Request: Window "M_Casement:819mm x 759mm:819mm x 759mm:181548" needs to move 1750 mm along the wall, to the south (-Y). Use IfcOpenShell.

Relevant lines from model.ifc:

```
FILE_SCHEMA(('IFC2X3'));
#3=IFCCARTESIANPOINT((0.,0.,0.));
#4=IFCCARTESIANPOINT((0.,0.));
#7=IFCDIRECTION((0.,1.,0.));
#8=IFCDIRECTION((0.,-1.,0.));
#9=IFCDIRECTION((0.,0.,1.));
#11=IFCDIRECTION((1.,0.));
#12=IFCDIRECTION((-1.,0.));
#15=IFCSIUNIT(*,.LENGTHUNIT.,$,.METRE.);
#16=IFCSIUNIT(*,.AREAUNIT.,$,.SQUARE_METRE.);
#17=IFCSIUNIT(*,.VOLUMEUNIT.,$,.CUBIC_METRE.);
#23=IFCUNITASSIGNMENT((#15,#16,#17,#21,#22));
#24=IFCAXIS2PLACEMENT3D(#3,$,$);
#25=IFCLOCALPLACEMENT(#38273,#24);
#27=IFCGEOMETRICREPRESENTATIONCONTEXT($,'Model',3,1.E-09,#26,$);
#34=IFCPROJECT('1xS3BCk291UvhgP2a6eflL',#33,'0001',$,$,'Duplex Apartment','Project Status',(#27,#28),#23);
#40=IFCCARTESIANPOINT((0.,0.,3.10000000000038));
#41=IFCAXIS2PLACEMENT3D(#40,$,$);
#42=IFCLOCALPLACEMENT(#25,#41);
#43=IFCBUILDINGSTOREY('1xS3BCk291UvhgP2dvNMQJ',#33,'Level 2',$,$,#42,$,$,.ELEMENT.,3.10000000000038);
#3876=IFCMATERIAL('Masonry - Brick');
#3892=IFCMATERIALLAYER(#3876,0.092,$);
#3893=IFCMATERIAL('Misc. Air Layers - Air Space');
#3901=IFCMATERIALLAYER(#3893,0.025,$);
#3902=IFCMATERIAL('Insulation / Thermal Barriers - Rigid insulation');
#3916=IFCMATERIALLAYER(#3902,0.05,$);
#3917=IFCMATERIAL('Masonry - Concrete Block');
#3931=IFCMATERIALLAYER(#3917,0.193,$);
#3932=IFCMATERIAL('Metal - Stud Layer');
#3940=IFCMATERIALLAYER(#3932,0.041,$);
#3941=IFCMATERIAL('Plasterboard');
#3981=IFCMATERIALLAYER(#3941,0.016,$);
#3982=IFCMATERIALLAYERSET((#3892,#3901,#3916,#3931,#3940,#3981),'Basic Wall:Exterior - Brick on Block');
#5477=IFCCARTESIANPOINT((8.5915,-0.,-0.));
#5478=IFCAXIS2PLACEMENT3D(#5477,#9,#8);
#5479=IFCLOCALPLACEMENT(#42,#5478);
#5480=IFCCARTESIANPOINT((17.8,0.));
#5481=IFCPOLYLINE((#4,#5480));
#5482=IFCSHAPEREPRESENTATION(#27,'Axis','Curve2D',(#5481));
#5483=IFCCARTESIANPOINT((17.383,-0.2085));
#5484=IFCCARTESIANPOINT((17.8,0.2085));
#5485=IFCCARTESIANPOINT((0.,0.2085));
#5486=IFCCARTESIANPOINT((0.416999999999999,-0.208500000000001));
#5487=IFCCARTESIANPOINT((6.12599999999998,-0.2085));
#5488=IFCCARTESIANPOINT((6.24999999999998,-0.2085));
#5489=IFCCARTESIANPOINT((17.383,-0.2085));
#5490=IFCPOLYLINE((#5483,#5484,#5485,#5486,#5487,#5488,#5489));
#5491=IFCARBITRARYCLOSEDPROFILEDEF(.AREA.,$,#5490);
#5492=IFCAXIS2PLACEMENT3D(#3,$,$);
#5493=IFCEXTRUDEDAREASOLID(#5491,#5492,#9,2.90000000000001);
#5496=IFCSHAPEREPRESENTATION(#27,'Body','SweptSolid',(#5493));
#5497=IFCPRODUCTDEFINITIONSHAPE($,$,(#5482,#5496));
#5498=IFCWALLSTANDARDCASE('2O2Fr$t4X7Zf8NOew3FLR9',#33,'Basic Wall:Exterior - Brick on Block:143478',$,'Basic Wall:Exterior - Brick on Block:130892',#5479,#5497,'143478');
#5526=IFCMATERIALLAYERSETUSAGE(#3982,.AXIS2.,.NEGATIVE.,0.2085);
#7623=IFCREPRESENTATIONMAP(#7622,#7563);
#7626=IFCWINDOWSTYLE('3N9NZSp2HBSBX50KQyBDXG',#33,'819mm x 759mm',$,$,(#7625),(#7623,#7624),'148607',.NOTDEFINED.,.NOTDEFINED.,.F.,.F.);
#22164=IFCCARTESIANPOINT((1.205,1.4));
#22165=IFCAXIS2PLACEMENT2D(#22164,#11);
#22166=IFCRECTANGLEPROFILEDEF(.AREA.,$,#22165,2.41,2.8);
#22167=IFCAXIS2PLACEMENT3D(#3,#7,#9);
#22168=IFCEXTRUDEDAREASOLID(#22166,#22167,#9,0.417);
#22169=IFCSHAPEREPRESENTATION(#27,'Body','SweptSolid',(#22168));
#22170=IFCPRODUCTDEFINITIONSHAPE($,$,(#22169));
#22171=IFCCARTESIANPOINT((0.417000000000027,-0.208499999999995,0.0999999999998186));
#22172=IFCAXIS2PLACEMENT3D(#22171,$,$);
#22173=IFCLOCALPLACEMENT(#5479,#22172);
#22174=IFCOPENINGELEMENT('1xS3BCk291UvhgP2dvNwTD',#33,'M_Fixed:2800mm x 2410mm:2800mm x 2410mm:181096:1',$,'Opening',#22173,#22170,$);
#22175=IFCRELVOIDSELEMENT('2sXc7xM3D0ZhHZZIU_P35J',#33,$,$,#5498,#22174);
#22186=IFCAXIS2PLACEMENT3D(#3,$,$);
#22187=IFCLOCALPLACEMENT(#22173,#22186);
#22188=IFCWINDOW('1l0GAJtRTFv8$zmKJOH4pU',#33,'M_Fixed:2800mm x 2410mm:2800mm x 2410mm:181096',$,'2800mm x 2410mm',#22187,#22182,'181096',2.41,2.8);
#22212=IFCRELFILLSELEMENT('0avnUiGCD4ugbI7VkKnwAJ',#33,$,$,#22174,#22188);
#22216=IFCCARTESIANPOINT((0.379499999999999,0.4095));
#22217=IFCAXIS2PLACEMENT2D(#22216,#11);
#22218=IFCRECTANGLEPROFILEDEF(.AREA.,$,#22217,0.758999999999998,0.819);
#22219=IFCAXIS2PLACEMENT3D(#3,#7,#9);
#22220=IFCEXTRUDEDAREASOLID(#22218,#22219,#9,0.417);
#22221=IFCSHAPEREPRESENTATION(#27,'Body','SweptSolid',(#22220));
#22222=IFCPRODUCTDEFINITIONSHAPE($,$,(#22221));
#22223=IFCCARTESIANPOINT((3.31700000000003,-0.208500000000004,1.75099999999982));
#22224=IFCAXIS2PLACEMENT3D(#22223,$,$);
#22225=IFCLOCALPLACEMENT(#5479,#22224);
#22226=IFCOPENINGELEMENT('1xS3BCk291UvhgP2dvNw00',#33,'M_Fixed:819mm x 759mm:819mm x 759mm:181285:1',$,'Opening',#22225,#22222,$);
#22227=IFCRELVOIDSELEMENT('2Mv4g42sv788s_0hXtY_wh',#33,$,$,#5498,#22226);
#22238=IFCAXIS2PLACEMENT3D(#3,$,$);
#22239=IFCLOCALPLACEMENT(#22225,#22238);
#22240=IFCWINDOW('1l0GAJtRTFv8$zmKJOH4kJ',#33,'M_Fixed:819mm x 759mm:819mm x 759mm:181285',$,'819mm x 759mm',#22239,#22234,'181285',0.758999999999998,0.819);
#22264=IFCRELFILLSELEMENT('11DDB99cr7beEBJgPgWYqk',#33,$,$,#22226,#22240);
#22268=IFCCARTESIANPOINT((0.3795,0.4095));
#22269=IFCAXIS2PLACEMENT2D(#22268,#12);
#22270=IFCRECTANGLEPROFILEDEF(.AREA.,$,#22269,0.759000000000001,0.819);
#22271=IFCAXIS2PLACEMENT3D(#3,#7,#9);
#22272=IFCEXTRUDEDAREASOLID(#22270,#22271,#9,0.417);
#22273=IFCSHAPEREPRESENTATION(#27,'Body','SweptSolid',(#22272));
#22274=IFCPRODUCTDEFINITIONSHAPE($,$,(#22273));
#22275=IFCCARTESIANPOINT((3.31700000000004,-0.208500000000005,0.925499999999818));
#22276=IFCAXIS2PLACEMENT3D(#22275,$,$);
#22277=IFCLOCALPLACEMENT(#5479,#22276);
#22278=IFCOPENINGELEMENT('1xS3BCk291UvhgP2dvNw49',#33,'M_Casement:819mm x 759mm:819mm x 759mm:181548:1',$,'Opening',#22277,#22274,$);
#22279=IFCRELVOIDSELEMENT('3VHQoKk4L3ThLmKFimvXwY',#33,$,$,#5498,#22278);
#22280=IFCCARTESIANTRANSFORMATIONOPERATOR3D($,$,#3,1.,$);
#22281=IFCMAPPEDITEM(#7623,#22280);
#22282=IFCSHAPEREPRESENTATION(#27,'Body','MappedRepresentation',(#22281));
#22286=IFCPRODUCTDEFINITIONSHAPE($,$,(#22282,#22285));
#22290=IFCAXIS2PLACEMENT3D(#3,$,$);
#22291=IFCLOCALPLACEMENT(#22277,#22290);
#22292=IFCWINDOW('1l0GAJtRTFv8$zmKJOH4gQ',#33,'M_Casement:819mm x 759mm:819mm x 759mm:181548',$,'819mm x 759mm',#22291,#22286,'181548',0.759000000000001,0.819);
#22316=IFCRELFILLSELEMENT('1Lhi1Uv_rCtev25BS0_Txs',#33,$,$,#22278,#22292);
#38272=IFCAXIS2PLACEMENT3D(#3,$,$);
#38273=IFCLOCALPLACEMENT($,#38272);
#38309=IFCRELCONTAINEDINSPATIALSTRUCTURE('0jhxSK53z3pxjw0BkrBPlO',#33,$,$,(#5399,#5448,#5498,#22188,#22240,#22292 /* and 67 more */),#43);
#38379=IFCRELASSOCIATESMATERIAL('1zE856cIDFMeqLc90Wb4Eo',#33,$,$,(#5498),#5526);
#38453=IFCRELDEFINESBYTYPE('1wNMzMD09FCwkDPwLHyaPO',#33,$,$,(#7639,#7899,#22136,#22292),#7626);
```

```python
import ifcopenshell
import ifcopenshell.api.geometry
import ifcopenshell.util.placement
import ifcopenshell.util.unit

model = ifcopenshell.open("model.ifc")
unit_scale = ifcopenshell.util.unit.calculate_unit_scale(model)

window = model.by_guid("1l0GAJtRTFv8$zmKJOH4gQ")
opening = window.FillsVoids[0].RelatingOpeningElement
wall = opening.VoidsElements[0].RelatingBuildingElement

wall_matrix = ifcopenshell.util.placement.get_local_placement(wall.ObjectPlacement)
shift = wall_matrix[:3, 0] * 1.75 / unit_scale
before = ifcopenshell.util.placement.get_local_placement(window.ObjectPlacement)[:3, 3].copy()

# The window is placed relative to its opening, so it follows when the opening moves.
matrix = ifcopenshell.util.placement.get_local_placement(opening.ObjectPlacement)
matrix[:3, 3] += shift
ifcopenshell.api.geometry.edit_object_placement(
    model, product=opening, matrix=matrix, is_si=False, should_transform_children=True
)

after = ifcopenshell.util.placement.get_local_placement(window.ObjectPlacement)[:3, 3]
print("window moved by", (after - before).round(3) + 0.0)

model.write("model_updated.ifc")
```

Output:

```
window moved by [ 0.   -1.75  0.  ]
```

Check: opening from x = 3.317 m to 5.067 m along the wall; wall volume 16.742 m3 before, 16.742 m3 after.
